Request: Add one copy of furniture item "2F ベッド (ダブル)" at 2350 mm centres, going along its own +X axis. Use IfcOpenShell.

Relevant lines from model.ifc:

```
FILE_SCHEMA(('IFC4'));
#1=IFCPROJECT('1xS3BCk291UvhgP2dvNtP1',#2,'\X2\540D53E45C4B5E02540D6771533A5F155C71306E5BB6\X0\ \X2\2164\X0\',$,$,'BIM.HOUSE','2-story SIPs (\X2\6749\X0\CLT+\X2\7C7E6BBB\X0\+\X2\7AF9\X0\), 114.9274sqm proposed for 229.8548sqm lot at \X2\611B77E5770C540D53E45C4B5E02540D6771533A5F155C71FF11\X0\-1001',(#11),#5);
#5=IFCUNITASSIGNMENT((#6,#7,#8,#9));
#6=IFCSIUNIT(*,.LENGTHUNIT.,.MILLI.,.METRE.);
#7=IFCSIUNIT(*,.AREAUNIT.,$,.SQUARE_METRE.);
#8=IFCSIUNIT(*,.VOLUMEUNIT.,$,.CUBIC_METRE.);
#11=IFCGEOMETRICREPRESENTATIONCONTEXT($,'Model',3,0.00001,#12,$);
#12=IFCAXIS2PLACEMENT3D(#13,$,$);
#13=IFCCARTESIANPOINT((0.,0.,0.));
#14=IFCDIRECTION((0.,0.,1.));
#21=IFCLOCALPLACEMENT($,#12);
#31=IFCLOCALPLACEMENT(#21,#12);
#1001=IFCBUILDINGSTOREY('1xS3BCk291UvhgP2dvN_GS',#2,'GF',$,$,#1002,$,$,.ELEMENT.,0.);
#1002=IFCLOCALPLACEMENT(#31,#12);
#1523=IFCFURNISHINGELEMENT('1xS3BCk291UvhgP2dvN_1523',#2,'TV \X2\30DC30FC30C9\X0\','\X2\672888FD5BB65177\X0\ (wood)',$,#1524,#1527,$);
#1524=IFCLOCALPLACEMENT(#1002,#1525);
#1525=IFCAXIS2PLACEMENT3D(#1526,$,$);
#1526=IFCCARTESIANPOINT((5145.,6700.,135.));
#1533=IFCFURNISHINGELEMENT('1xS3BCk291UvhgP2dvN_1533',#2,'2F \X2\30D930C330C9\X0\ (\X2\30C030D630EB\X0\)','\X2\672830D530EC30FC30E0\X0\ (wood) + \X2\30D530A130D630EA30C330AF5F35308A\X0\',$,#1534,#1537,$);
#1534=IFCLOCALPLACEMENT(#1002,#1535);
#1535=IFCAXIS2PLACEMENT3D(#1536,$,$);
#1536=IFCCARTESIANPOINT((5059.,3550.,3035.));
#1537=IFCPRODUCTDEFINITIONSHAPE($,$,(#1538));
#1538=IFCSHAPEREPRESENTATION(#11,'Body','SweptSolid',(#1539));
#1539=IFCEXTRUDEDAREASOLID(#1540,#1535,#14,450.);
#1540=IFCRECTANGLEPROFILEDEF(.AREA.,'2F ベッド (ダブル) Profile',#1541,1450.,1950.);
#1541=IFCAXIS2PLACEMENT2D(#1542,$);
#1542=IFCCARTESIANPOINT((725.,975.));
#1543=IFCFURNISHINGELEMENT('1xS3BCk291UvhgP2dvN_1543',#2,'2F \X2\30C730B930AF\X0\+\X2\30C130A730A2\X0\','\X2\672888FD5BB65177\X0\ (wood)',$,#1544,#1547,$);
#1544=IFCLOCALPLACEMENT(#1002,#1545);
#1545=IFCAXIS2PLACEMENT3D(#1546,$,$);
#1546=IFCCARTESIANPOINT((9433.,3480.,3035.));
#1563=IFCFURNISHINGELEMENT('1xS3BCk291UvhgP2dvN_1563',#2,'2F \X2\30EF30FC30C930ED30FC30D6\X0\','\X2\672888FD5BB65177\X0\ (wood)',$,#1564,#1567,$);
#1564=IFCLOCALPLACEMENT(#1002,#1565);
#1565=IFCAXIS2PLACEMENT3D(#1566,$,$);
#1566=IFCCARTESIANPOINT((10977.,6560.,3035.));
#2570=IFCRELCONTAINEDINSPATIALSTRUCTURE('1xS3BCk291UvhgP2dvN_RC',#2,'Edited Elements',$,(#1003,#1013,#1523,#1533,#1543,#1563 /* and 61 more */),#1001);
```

```python
import ifcopenshell
import ifcopenshell.api.geometry
import ifcopenshell.api.root
import ifcopenshell.util.element
import ifcopenshell.util.placement
import ifcopenshell.util.unit

model = ifcopenshell.open("model.ifc")
unit_scale = ifcopenshell.util.unit.calculate_unit_scale(model)


def reuse_history(source, copy):
    """copy_class also copies each property set's owner history, people and application; keep the originals."""
    for rel in copy.IsDefinedBy:
        if rel.is_a("IfcRelDefinesByProperties") and (history := rel.RelatingPropertyDefinition.OwnerHistory):
            rel.RelatingPropertyDefinition.OwnerHistory = source.OwnerHistory
            ifcopenshell.util.element.remove_deep2(model, history)


source = model.by_guid("1xS3BCk291UvhgP2dvN_1533")
base = ifcopenshell.util.placement.get_local_placement(source.ObjectPlacement)
step = base[:3, 0] * 2.35 / unit_scale

for i in range(1, 2):
    copy = ifcopenshell.api.root.copy_class(model, product=source)
    copy.Representation = ifcopenshell.util.element.copy_deep(
        model, source.Representation, exclude=["IfcGeometricRepresentationContext", "IfcRepresentationMap"]
    )
    reuse_history(source, copy)
    matrix = base.copy()
    matrix[:3, 3] += i * step
    print("added at", matrix[:3, 3].round(3) + 0.0)
    ifcopenshell.api.geometry.edit_object_placement(model, product=copy, matrix=matrix, is_si=False)

model.write("model-out.ifc")
```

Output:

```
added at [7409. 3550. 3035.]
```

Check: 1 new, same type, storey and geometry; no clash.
